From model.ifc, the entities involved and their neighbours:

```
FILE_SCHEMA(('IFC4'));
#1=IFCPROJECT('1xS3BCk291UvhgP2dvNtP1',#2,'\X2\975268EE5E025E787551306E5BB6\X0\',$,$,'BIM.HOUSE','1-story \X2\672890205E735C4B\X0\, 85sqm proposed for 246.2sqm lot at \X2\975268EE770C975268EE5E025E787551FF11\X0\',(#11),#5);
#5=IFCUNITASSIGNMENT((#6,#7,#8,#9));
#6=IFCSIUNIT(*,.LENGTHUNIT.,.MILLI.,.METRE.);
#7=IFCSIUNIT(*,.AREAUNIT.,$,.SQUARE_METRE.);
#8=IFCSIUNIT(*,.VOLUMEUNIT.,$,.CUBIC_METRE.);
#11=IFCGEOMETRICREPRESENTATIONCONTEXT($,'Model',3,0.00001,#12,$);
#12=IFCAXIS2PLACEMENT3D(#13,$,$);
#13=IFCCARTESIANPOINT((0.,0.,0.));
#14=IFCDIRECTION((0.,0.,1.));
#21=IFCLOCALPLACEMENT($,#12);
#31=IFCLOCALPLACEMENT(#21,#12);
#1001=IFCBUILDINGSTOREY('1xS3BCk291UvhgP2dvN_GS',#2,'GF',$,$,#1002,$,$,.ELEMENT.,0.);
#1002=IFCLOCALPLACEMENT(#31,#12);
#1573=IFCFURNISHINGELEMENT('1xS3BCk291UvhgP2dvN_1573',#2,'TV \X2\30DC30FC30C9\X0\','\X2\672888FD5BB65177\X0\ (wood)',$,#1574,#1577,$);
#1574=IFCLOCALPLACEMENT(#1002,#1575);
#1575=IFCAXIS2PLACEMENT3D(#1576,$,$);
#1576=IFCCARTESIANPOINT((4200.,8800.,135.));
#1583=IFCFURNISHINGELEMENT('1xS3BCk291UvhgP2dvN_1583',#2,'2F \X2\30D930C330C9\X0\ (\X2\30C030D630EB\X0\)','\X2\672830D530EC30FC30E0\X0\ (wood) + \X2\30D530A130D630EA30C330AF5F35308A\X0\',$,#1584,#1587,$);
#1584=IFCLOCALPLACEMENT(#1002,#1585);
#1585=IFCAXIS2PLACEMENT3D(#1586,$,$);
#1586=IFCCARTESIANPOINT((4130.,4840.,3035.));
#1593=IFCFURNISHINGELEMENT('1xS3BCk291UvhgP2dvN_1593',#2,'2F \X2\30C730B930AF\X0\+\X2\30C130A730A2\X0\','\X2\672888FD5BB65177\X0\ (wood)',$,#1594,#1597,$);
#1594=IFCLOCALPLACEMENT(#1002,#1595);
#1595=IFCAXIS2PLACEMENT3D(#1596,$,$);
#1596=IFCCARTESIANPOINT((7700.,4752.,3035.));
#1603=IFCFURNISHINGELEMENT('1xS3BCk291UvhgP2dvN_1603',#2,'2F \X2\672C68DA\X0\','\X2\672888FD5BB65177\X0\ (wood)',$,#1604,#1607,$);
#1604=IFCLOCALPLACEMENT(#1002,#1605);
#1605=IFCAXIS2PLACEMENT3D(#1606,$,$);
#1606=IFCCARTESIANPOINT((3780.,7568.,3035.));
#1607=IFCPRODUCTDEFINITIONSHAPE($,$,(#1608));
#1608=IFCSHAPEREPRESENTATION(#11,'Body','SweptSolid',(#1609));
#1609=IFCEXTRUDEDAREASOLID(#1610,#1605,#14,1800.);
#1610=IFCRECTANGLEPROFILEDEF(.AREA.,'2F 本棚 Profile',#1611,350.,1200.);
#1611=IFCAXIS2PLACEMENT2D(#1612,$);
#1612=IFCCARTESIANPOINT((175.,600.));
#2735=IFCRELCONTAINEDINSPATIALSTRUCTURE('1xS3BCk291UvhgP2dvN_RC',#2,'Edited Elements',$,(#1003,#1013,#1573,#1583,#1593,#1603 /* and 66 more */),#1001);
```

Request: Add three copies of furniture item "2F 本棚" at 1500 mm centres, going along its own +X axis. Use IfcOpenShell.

```python
import ifcopenshell
import ifcopenshell.api.geometry
import ifcopenshell.api.root
import ifcopenshell.util.element
import ifcopenshell.util.placement
import ifcopenshell.util.unit

model = ifcopenshell.open("model.ifc")
unit_scale = ifcopenshell.util.unit.calculate_unit_scale(model)


def reuse_history(source, copy):
    """copy_class also copies each property set's owner history, people and application; keep the originals."""
    for rel in copy.IsDefinedBy:
        if rel.is_a("IfcRelDefinesByProperties") and (history := rel.RelatingPropertyDefinition.OwnerHistory):
            rel.RelatingPropertyDefinition.OwnerHistory = source.OwnerHistory
            ifcopenshell.util.element.remove_deep2(model, history)


source = model.by_guid("1xS3BCk291UvhgP2dvN_1603")
base = ifcopenshell.util.placement.get_local_placement(source.ObjectPlacement)
step = base[:3, 0] * 1.5 / unit_scale

for i in range(1, 4):
    copy = ifcopenshell.api.root.copy_class(model, product=source)
    copy.Representation = ifcopenshell.util.element.copy_deep(
        model, source.Representation, exclude=["IfcGeometricRepresentationContext", "IfcRepresentationMap"]
    )
    reuse_history(source, copy)
    matrix = base.copy()
    matrix[:3, 3] += i * step
    print("added at", matrix[:3, 3].round(3) + 0.0)
    ifcopenshell.api.geometry.edit_object_placement(model, product=copy, matrix=matrix, is_si=False)

model.write("model_rev.ifc")
```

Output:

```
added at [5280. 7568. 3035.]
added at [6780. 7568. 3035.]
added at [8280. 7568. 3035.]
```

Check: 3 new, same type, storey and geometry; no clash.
